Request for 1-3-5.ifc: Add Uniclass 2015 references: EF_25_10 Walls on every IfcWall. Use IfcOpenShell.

First a look at what the model holds.

```python
import ifcopenshell

model = ifcopenshell.open("1-3-5.ifc")
print(model.schema)
print("classifications:", [c.Name for c in model.by_type("IfcClassification")])
for ifc_class in ("IfcDoor", "IfcRoof", "IfcStair", "IfcWall", "IfcWindow"):
    print(ifc_class, len(model.by_type(ifc_class)))
```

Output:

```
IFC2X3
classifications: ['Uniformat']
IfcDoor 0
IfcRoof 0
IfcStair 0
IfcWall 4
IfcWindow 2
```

```python
import ifcopenshell
import ifcopenshell.api.classification

model = ifcopenshell.open("1-3-5.ifc")

# IFC2X3 requires Source and Edition and has no link from the project to the system.
system = model.create_entity("IfcClassification", Source="NBS", Edition="2015", Name="Uniclass 2015")

codes = {
    "IfcWall": ("EF_25_10", "Walls"),
}
for ifc_class, (code, name) in codes.items():
    products = model.by_type(ifc_class)
    ifcopenshell.api.classification.add_reference(
        model, products=products, classification=system, identification=code, name=name
    )
    print(code, len(products))

model.write("1-3-5_edited.ifc")
```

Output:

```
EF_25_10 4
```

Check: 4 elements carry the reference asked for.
